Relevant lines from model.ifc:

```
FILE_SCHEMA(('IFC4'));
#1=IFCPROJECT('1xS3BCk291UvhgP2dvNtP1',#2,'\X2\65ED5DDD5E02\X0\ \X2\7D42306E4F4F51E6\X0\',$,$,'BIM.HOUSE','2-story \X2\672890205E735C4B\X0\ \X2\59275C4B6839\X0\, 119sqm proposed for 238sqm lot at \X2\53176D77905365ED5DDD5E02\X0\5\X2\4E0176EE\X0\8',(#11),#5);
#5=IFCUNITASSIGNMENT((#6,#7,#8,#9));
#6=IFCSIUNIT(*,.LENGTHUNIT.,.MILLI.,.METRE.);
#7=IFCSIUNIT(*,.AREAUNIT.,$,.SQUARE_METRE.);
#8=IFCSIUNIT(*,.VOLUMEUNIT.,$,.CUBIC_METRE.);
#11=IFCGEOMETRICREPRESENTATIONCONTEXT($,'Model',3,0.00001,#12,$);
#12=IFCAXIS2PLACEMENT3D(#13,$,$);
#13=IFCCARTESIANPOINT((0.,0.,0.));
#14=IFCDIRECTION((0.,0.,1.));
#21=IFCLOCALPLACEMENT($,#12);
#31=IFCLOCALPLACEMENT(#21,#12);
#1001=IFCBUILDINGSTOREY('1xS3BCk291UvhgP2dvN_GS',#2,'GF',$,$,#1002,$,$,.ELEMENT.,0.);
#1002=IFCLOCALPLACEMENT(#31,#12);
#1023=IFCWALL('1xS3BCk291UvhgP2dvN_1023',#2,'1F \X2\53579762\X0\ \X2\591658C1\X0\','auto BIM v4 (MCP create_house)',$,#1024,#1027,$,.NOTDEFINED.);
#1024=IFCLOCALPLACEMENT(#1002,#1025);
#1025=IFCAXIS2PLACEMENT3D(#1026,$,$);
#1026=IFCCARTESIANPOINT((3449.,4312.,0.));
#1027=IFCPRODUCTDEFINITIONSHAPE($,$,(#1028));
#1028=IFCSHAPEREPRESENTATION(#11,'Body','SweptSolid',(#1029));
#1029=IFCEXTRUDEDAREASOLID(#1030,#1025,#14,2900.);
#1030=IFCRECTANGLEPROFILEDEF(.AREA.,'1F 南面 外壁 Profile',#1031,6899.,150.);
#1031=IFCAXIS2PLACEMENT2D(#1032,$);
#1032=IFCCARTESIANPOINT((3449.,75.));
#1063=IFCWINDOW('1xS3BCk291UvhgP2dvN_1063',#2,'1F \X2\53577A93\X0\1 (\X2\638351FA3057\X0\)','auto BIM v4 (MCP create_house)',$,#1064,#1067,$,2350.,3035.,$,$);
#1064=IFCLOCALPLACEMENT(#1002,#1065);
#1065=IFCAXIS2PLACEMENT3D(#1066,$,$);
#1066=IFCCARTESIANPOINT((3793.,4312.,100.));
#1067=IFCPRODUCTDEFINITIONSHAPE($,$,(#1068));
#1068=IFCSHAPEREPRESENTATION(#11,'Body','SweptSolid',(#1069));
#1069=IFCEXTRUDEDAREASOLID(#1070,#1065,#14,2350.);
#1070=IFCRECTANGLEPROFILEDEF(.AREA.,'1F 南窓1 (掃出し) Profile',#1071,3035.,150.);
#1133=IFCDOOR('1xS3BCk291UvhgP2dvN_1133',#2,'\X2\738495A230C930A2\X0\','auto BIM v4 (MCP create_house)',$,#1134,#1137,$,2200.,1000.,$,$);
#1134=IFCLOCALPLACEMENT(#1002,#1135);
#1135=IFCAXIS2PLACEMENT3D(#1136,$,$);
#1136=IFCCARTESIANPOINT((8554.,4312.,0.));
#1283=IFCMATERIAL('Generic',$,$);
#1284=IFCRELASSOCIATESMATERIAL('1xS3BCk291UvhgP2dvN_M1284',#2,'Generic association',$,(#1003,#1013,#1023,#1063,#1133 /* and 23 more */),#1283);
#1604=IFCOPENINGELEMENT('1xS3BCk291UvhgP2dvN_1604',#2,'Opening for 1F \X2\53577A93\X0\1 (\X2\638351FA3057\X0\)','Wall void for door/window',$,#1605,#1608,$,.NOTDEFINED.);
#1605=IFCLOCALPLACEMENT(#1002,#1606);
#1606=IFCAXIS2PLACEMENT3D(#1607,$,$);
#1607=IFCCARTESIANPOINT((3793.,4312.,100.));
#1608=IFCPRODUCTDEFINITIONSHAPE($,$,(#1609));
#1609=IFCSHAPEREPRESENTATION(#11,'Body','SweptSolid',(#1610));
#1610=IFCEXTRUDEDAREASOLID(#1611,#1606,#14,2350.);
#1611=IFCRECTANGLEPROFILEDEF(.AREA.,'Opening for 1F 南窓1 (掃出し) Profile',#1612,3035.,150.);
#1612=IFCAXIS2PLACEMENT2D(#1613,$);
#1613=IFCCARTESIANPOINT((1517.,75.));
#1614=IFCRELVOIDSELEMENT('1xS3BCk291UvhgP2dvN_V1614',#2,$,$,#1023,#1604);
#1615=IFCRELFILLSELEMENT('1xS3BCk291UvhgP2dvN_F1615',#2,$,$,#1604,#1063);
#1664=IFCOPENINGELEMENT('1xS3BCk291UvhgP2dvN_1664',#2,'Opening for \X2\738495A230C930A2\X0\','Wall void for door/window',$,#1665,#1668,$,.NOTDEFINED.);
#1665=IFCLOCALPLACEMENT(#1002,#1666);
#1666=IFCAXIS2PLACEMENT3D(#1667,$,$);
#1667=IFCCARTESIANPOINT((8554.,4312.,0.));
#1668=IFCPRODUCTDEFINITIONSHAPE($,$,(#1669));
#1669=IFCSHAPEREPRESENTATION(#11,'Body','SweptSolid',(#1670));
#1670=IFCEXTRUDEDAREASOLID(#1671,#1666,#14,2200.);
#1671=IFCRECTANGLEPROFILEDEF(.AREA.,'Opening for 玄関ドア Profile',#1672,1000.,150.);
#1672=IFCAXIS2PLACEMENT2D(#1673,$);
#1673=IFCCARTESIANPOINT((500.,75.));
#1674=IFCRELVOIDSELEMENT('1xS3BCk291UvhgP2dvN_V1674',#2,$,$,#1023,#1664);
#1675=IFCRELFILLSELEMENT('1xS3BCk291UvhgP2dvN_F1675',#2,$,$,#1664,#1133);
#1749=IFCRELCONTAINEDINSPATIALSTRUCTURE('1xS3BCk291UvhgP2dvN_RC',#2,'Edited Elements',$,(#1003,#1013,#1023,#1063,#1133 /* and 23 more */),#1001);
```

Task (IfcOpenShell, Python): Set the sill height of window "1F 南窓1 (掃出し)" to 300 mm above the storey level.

```python
import numpy as np
import ifcopenshell
import ifcopenshell.api.geometry
import ifcopenshell.geom
import ifcopenshell.util.element
import ifcopenshell.util.placement
import ifcopenshell.util.shape
import ifcopenshell.util.unit

model = ifcopenshell.open("model.ifc")
unit_scale = ifcopenshell.util.unit.calculate_unit_scale(model)

window = model.by_guid("1xS3BCk291UvhgP2dvN_1063")
opening = window.FillsVoids[0].RelatingOpeningElement
storey = ifcopenshell.util.element.get_container(window, ifc_class="IfcBuildingStorey")
level = ifcopenshell.util.placement.get_local_placement(storey.ObjectPlacement)[2, 3]

# The opening's origin need not be at the sill, so measure its lowest point.
shape = ifcopenshell.geom.create_shape(ifcopenshell.geom.settings(), opening)
bottom = ifcopenshell.util.shape.get_shape_bottom_elevation(shape, shape.geometry) / unit_scale
dz = level + 0.3 / unit_scale - bottom

shift = np.array([0.0, 0.0, dz])
# The window is not placed relative to its opening, so move both.
for product in (opening, window):
    matrix = ifcopenshell.util.placement.get_local_placement(product.ObjectPlacement)
    matrix[:3, 3] += shift
    ifcopenshell.api.geometry.edit_object_placement(model, product=product, matrix=matrix, is_si=False)

print(f"moved by {dz * unit_scale:+.3f} m")

model.write("model_rev.ifc")
```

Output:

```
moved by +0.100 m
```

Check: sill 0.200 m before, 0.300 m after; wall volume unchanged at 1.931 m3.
